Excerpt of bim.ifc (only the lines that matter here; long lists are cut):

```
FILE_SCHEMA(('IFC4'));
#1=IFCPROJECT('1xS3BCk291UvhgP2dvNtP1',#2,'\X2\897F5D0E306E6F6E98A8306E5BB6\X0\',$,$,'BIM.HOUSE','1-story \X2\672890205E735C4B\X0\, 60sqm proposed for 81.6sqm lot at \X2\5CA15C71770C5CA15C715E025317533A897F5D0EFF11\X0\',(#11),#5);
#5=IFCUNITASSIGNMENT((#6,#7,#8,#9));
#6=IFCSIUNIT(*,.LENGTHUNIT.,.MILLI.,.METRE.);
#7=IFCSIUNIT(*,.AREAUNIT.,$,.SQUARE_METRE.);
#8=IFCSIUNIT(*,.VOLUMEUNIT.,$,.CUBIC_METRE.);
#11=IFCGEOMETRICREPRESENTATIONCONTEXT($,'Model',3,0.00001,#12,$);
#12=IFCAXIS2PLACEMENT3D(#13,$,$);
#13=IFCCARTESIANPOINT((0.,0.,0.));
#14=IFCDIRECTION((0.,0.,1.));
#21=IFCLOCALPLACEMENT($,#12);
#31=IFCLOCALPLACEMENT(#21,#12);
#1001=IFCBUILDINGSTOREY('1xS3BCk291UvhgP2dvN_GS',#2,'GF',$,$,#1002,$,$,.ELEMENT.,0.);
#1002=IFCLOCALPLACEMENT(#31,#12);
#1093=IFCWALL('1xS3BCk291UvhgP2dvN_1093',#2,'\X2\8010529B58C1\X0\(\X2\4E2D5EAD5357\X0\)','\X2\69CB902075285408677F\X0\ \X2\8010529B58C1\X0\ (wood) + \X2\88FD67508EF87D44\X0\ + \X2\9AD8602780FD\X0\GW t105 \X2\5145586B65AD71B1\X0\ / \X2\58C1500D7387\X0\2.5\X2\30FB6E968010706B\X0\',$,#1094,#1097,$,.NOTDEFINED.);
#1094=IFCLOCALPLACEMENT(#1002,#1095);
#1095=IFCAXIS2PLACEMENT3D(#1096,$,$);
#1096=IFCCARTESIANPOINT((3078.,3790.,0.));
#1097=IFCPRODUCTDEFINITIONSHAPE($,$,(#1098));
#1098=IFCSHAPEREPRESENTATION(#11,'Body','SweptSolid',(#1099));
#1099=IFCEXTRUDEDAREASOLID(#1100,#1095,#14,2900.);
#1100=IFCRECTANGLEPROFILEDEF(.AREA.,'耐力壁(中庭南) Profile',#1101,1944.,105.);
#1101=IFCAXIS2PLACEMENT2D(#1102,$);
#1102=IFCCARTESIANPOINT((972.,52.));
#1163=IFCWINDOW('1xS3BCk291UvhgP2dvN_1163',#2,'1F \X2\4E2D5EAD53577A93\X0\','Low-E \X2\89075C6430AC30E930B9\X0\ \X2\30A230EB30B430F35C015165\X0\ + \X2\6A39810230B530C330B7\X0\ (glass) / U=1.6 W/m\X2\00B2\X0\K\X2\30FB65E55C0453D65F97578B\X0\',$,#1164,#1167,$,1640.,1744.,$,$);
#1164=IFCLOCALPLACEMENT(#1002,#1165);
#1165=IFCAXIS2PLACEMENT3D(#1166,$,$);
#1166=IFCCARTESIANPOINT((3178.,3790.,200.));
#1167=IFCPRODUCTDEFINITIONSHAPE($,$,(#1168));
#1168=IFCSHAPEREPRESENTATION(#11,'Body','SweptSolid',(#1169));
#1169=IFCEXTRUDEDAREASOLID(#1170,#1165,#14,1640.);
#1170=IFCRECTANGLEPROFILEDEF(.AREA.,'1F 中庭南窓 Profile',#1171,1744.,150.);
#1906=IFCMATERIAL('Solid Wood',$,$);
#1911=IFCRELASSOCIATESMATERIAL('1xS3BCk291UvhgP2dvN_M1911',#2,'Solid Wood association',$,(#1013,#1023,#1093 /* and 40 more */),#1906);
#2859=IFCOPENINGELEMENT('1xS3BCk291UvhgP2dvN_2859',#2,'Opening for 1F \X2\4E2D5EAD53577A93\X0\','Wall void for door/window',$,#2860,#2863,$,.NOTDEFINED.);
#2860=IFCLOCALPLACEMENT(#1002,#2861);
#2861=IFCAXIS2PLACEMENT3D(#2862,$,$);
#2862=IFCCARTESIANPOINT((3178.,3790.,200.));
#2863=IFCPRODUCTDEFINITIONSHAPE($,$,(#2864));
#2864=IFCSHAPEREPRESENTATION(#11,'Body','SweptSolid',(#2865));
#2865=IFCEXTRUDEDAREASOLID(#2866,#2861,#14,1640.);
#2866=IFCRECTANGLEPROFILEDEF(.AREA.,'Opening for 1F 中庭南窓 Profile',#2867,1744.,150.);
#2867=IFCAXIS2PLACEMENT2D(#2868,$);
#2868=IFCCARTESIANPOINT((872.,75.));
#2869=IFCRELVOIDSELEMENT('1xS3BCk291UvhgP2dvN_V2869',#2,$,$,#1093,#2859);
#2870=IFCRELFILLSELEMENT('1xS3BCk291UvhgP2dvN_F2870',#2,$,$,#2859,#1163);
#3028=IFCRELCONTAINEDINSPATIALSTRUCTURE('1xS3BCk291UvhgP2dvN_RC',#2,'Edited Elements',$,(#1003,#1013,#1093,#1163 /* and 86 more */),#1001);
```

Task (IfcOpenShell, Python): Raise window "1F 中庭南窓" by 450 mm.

```python
import numpy as np
import ifcopenshell
import ifcopenshell.api.geometry
import ifcopenshell.util.placement
import ifcopenshell.util.unit

model = ifcopenshell.open("bim.ifc")
unit_scale = ifcopenshell.util.unit.calculate_unit_scale(model)

window = model.by_id(1163)
opening = window.FillsVoids[0].RelatingOpeningElement
dz = 0.45 / unit_scale

shift = np.array([0.0, 0.0, dz])
# The window is not placed relative to its opening, so move both.
for product in (opening, window):
    matrix = ifcopenshell.util.placement.get_local_placement(product.ObjectPlacement)
    matrix[:3, 3] += shift
    ifcopenshell.api.geometry.edit_object_placement(model, product=product, matrix=matrix, is_si=False)

print(f"moved by {dz * unit_scale:+.3f} m")

model.write("bim-out.ifc")
```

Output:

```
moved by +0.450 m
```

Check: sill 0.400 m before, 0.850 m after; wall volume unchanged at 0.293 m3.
